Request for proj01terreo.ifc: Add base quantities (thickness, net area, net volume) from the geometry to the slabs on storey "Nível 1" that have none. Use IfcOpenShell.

First a look at what the model holds.

```python
import ifcopenshell
import ifcopenshell.util.element
import ifcopenshell.util.unit

model = ifcopenshell.open("proj01terreo.ifc")
print(model.schema)
for unit_type in ("LENGTHUNIT", "AREAUNIT", "VOLUMEUNIT"):
    print(unit_type, ifcopenshell.util.unit.calculate_unit_scale(model, unit_type))
storey = next(s for s in model.by_type("IfcBuildingStorey") if s.Name == "Nível 1")
slabs = [e for e in ifcopenshell.util.element.get_decomposition(storey) if e.is_a("IfcSlab")]
for e in sorted(slabs, key=lambda e: e.id()):
    print(e.id(), e.is_a(), e.Name, list(ifcopenshell.util.element.get_psets(e, qtos_only=True)), sep=" | ")
```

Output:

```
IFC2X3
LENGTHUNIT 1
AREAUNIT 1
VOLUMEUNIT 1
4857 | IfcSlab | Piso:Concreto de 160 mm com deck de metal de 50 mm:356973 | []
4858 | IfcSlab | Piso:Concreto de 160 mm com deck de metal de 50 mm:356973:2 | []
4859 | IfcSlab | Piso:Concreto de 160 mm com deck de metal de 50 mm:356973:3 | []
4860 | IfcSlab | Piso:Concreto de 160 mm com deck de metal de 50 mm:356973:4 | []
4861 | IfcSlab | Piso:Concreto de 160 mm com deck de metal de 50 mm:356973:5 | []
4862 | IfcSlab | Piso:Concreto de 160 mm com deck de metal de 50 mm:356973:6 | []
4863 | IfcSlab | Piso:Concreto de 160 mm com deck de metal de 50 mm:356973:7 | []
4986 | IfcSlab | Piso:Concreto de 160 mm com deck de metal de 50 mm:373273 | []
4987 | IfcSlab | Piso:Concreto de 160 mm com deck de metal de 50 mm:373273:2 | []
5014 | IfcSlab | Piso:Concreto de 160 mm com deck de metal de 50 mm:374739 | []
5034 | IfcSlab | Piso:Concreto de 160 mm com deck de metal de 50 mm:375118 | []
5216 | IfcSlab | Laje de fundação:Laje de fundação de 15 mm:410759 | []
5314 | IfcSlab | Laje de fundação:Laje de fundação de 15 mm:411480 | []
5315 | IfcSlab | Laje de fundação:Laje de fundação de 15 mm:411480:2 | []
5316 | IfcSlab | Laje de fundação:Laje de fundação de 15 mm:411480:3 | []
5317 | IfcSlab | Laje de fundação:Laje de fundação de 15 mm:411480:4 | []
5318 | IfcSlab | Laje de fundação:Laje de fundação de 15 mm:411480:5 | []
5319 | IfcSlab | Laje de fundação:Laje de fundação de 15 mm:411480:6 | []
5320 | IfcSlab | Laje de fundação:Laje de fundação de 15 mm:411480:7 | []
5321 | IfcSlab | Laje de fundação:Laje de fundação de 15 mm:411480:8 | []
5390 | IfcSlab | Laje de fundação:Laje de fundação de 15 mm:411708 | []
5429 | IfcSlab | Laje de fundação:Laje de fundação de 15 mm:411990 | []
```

```python
import ifcopenshell
import ifcopenshell.api.pset
import ifcopenshell.geom
import ifcopenshell.util.element
import ifcopenshell.util.shape
import ifcopenshell.util.unit

model = ifcopenshell.open("proj01terreo.ifc")
unit_scale = ifcopenshell.util.unit.calculate_unit_scale(model)
area_scale = ifcopenshell.util.unit.calculate_unit_scale(model, "AREAUNIT")
volume_scale = ifcopenshell.util.unit.calculate_unit_scale(model, "VOLUMEUNIT")
settings = ifcopenshell.geom.settings()

storey = next(s for s in model.by_type("IfcBuildingStorey") if s.Name == "Nível 1")
slabs = [e for e in ifcopenshell.util.element.get_decomposition(storey) if e.is_a("IfcSlab")]

for e in sorted(slabs, key=lambda e: e.id()):
    if ifcopenshell.util.element.get_psets(e, qtos_only=True, should_inherit=False):
        continue
    # Geometry comes back in metres, in the element's own axes.
    shape = ifcopenshell.geom.create_shape(settings, e)
    values = {
        "Width": ifcopenshell.util.shape.get_z(shape.geometry) / unit_scale,
        "NetArea": ifcopenshell.util.shape.get_footprint_area(shape.geometry) / area_scale,
        "NetVolume": ifcopenshell.util.shape.get_volume(shape.geometry) / volume_scale,
    }
    qto = ifcopenshell.api.pset.add_qto(model, product=e, name="BaseQuantities")
    ifcopenshell.api.pset.edit_qto(model, qto=qto, properties=values)
    print(e.id(), {k: round(v, 3) for k, v in values.items()})

model.write("proj01terreo-out.ifc")
```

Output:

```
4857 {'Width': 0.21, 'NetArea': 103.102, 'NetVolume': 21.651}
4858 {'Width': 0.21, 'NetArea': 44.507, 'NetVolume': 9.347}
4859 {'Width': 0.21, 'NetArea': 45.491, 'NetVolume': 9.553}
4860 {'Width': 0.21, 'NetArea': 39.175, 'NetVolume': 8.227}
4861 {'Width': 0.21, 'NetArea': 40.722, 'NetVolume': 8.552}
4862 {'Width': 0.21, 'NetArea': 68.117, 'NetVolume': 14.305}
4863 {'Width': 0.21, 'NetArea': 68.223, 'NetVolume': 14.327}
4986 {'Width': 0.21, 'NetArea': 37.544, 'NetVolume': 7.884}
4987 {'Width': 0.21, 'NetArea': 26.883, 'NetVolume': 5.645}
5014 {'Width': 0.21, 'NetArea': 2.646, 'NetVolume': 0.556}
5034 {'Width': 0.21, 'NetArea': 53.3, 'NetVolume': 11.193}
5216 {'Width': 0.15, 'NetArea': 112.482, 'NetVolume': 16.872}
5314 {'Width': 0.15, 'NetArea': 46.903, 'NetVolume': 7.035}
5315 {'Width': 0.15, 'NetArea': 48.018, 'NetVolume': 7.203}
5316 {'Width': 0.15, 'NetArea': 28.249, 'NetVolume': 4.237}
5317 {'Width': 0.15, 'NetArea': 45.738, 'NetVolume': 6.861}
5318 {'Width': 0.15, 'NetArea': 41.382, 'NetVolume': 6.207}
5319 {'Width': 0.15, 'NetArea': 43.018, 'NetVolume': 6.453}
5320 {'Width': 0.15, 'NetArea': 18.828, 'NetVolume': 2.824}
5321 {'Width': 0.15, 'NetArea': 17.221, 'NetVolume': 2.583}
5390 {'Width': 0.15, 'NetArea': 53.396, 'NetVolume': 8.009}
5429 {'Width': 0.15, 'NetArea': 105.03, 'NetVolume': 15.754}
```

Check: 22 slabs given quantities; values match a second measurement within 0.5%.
